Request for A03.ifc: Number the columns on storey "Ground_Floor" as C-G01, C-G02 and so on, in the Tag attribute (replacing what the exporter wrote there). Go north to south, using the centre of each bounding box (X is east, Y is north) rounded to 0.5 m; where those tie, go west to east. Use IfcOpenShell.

First a look at what the model holds.

```python
import ifcopenshell
import ifcopenshell.util.element
import ifcopenshell.util.placement

model = ifcopenshell.open("A03.ifc")
print(model.schema)
storey = next(s for s in model.by_type("IfcBuildingStorey") if s.Name == "Ground_Floor")
columns = [e for e in ifcopenshell.util.element.get_decomposition(storey) if e.is_a("IfcColumn")]
for e in sorted(columns, key=lambda e: e.id()):
    origin = ifcopenshell.util.placement.get_local_placement(e.ObjectPlacement)[:3, 3]
    print(e.id(), e.Tag, e.Name, origin.round(2) + 0.0, sep=" | ")
```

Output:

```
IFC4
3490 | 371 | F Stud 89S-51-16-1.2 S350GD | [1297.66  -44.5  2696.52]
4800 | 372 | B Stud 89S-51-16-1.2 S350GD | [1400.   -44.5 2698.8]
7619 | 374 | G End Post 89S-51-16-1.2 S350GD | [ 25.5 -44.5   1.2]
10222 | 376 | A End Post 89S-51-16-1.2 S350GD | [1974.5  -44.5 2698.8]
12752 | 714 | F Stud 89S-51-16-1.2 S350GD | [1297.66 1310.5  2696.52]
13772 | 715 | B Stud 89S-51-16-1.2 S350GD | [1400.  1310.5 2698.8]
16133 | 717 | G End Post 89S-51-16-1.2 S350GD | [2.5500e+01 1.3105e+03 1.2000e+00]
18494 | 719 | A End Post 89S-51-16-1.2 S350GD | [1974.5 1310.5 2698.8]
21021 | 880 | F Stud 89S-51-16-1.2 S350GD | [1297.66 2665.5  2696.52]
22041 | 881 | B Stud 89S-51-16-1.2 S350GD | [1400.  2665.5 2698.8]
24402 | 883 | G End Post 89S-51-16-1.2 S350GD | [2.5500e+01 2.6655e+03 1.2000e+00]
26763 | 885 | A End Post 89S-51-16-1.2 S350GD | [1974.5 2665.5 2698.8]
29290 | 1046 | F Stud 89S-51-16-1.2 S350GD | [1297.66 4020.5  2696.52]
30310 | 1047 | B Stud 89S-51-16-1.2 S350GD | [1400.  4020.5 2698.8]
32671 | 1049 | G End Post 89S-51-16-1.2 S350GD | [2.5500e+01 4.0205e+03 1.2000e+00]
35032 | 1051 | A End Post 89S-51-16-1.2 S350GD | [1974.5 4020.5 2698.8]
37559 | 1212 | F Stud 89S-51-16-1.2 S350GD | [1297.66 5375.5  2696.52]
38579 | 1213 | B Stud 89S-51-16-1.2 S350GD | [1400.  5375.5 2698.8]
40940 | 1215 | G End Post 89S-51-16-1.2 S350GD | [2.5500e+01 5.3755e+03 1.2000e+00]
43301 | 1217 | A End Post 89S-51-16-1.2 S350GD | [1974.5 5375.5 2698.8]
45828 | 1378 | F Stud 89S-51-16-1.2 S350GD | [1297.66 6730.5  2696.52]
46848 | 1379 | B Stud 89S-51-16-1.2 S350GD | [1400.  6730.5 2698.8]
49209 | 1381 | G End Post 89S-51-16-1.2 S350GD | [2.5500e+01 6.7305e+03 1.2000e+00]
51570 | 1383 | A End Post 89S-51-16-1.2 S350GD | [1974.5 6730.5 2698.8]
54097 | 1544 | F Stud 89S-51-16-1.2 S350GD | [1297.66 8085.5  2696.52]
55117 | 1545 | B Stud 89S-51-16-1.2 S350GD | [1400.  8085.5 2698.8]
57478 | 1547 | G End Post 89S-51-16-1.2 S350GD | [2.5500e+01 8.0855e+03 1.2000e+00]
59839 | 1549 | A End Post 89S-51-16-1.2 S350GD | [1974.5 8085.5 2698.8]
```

```python
import ifcopenshell
import ifcopenshell.geom
import ifcopenshell.util.element
import ifcopenshell.util.shape

model = ifcopenshell.open("A03.ifc")
settings = ifcopenshell.geom.settings()
settings.set("use-world-coords", True)


def centre(element):
    shape = ifcopenshell.geom.create_shape(settings, element)
    return ifcopenshell.util.shape.get_bbox_centroid(shape.geometry)


storey = next(s for s in model.by_type("IfcBuildingStorey") if s.Name == "Ground_Floor")
columns = [e for e in ifcopenshell.util.element.get_decomposition(storey) if e.is_a("IfcColumn")]

# Insertion points can sit at a corner or the storey origin, so sort by the geometry (in metres).
centres = {e: centre(e) for e in columns}
columns.sort(key=lambda e: (-round(centres[e][1] / 0.5), centres[e][0]))

for i, e in enumerate(columns, start=1):
    number = f"C-G{i:02d}"
    e.Tag = number
    print(e.id(), number)

model.write("A03_edited.ifc")
```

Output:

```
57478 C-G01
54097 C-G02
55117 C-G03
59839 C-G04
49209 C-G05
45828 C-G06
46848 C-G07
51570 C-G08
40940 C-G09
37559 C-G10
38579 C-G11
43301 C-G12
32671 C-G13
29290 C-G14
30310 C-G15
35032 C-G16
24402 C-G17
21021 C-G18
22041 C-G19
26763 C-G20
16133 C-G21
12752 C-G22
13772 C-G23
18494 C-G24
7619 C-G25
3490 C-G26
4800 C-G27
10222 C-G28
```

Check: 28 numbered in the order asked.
